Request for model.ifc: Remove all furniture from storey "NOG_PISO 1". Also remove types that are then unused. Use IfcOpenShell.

First a look at what the model holds.

```python
import ifcopenshell
import ifcopenshell.util.element

model = ifcopenshell.open("model.ifc")
print(model.schema)
storey = next(s for s in model.by_type("IfcBuildingStorey") if s.Name == "NOG_PISO 1")
furniture = [e for e in ifcopenshell.util.element.get_decomposition(storey) if e.is_a("IfcFurnishingElement")]
seen = {}
for e in furniture:
    element_type = ifcopenshell.util.element.get_type(e)
    name = element_type.Name if element_type not in (None, e) else None
    seen[name] = seen.get(name, 0) + 1
for name, count in sorted(seen.items(), key=str):
    print(count, "x", name)
```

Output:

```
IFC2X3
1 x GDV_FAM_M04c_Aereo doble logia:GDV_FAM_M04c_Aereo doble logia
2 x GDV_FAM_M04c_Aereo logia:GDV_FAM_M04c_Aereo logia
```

```python
import ifcopenshell
import ifcopenshell.api.root
import ifcopenshell.util.element

model = ifcopenshell.open("model.ifc")

storey = next(s for s in model.by_type("IfcBuildingStorey") if s.Name == "NOG_PISO 1")
furniture = [e for e in ifcopenshell.util.element.get_decomposition(storey) if e.is_a("IfcFurnishingElement")]
types = {ifcopenshell.util.element.get_type(e) for e in furniture} - {None, *furniture}

for e in furniture:
    ifcopenshell.api.root.remove_product(model, product=e)
print(len(furniture), "removed")

unused = [t for t in types if not ifcopenshell.util.element.get_types(t)]
for t in unused:
    ifcopenshell.api.root.remove_product(model, product=t)
print(len(unused), "unused types removed")

model.write("model_rev.ifc")
```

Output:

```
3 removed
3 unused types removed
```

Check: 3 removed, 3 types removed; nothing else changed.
